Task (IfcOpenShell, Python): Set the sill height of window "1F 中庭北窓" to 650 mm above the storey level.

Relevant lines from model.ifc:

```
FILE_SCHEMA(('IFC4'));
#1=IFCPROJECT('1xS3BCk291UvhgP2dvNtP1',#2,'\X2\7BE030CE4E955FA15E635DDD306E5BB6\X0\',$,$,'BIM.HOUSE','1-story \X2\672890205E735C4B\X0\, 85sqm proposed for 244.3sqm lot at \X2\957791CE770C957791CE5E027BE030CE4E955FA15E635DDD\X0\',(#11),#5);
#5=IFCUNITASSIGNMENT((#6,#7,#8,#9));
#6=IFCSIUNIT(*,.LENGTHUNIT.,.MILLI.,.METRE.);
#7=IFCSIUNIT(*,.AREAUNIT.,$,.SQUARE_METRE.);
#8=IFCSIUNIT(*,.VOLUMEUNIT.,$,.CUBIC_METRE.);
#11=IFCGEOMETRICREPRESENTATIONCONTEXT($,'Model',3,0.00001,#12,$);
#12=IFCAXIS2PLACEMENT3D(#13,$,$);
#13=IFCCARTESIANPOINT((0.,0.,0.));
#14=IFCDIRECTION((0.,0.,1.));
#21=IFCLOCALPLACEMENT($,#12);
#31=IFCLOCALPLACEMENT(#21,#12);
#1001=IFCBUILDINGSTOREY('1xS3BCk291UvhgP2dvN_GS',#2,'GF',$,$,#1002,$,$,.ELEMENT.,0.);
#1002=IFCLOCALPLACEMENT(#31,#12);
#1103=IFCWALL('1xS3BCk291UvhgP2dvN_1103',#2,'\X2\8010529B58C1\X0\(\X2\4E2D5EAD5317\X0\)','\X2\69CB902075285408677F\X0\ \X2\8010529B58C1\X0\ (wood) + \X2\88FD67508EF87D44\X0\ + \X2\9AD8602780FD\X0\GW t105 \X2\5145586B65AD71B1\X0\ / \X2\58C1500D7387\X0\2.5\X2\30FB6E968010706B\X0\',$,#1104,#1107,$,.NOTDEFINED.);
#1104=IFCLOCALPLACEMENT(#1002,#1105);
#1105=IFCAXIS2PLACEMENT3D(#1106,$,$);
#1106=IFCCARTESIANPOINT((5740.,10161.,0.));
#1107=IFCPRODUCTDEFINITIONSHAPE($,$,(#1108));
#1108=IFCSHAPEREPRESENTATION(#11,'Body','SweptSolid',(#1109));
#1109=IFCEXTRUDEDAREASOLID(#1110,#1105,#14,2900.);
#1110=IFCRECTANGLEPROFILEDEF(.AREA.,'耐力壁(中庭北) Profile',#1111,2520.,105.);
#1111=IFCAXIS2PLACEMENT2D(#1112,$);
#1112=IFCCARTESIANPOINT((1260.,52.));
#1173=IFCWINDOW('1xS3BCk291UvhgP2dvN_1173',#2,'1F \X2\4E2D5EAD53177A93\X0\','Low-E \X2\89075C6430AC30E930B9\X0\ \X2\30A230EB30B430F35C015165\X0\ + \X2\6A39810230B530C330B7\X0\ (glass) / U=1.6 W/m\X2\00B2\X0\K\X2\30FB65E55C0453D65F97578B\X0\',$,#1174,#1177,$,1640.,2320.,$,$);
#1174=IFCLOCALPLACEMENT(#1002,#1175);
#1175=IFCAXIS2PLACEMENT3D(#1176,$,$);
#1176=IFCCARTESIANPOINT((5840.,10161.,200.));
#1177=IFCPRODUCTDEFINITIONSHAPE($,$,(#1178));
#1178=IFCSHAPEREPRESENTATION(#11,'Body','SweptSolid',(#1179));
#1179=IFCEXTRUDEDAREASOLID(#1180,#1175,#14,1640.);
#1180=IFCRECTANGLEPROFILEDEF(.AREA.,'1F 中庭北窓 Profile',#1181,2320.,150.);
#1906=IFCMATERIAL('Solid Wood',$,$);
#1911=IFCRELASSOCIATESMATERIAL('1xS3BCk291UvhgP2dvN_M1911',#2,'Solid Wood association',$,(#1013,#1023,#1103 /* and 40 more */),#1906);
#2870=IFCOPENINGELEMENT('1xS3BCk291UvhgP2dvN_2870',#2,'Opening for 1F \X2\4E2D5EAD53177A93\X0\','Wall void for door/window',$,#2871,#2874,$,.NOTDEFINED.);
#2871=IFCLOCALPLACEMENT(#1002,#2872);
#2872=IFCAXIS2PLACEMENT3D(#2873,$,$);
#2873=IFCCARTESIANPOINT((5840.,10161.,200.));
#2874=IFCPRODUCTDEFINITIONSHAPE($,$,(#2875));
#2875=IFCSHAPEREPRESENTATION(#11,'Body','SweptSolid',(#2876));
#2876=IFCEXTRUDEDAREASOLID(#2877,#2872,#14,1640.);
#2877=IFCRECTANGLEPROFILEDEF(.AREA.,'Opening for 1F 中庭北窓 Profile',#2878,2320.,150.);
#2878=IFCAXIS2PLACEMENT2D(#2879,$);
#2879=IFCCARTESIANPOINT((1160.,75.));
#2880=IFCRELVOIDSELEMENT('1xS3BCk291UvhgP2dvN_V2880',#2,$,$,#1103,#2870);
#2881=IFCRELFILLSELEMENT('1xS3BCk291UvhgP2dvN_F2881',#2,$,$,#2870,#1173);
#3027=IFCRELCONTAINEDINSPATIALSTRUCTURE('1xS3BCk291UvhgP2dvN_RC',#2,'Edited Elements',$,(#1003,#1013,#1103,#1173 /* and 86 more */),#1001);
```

```python
import numpy as np
import ifcopenshell
import ifcopenshell.api.geometry
import ifcopenshell.geom
import ifcopenshell.util.element
import ifcopenshell.util.placement
import ifcopenshell.util.shape
import ifcopenshell.util.unit

model = ifcopenshell.open("model.ifc")
unit_scale = ifcopenshell.util.unit.calculate_unit_scale(model)

window = model.by_id(1173)
opening = window.FillsVoids[0].RelatingOpeningElement
storey = ifcopenshell.util.element.get_container(window, ifc_class="IfcBuildingStorey")
level = ifcopenshell.util.placement.get_local_placement(storey.ObjectPlacement)[2, 3]

# The opening's origin need not be at the sill, so measure its lowest point.
shape = ifcopenshell.geom.create_shape(ifcopenshell.geom.settings(), opening)
bottom = ifcopenshell.util.shape.get_shape_bottom_elevation(shape, shape.geometry) / unit_scale
dz = level + 0.65 / unit_scale - bottom

shift = np.array([0.0, 0.0, dz])
# The window is not placed relative to its opening, so move both.
for product in (opening, window):
    matrix = ifcopenshell.util.placement.get_local_placement(product.ObjectPlacement)
    matrix[:3, 3] += shift
    ifcopenshell.api.geometry.edit_object_placement(model, product=product, matrix=matrix, is_si=False)

print(f"moved by {dz * unit_scale:+.3f} m")

model.write("model_rev.ifc")
```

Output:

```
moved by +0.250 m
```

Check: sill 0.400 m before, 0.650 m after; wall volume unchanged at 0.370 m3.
